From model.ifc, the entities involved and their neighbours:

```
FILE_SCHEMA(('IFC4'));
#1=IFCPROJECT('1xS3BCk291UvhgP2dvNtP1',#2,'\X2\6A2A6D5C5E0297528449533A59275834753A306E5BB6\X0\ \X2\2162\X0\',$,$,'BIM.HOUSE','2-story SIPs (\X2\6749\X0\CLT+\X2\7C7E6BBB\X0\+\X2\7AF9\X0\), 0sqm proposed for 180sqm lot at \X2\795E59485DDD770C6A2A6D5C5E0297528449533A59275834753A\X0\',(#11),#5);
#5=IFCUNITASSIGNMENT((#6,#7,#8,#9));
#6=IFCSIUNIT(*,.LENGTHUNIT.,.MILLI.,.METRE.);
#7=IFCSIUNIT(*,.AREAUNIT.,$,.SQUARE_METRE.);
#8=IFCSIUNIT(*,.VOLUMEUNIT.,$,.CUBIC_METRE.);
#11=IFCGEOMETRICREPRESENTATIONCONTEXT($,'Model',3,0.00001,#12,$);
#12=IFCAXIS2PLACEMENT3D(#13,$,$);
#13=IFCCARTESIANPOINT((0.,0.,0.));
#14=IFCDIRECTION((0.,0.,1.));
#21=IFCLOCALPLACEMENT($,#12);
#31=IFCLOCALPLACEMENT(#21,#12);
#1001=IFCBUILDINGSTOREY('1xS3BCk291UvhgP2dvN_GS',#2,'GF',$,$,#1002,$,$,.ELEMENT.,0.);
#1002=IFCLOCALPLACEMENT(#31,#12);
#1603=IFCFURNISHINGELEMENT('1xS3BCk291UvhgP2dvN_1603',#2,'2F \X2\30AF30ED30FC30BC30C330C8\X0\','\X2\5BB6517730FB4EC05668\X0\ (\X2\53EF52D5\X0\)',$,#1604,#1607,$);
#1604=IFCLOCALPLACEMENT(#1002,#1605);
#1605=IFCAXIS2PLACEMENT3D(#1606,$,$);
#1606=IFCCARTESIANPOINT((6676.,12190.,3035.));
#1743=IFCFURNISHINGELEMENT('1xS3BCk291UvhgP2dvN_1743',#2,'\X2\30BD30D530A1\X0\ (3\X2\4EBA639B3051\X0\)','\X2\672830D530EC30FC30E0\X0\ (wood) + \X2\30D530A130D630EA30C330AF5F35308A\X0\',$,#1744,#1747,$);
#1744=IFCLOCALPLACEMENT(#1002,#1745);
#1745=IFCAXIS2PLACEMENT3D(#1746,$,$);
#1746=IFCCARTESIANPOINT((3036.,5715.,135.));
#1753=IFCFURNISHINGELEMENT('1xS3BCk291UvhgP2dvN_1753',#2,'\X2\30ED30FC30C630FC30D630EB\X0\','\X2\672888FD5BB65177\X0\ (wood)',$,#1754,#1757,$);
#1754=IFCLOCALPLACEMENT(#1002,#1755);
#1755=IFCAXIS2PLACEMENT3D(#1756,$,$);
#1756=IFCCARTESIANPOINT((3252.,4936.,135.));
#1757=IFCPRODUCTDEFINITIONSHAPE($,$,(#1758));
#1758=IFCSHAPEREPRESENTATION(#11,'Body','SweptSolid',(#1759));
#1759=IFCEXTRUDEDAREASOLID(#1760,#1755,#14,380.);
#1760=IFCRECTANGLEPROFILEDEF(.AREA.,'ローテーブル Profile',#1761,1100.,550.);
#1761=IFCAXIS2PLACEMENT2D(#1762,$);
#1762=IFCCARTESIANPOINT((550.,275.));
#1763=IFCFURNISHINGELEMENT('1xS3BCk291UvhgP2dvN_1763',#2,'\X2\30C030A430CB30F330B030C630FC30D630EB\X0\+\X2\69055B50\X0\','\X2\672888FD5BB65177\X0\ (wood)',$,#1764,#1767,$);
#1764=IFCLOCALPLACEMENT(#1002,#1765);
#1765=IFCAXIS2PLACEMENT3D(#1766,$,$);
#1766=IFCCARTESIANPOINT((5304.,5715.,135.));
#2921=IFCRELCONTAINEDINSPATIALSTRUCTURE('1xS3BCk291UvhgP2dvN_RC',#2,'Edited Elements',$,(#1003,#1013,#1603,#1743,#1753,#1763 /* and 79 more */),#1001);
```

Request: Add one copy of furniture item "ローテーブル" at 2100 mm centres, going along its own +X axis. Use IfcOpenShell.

```python
import ifcopenshell
import ifcopenshell.api.geometry
import ifcopenshell.api.root
import ifcopenshell.util.element
import ifcopenshell.util.placement

model = ifcopenshell.open("model.ifc")


def reuse_history(source, copy):
    """copy_class also copies each property set's owner history, people and application; keep the originals."""
    for rel in copy.IsDefinedBy:
        if rel.is_a("IfcRelDefinesByProperties") and (history := rel.RelatingPropertyDefinition.OwnerHistory):
            rel.RelatingPropertyDefinition.OwnerHistory = source.OwnerHistory
            ifcopenshell.util.element.remove_deep2(model, history)


source = model.by_guid("1xS3BCk291UvhgP2dvN_1753")
base = ifcopenshell.util.placement.get_local_placement(source.ObjectPlacement)
step = base[:3, 0] * 2100.0

for i in range(1, 2):
    copy = ifcopenshell.api.root.copy_class(model, product=source)
    copy.Representation = ifcopenshell.util.element.copy_deep(
        model, source.Representation, exclude=["IfcGeometricRepresentationContext", "IfcRepresentationMap"]
    )
    reuse_history(source, copy)
    matrix = base.copy()
    matrix[:3, 3] += i * step
    print("added at", matrix[:3, 3].round(3) + 0.0)
    ifcopenshell.api.geometry.edit_object_placement(model, product=copy, matrix=matrix, is_si=False)

model.write("model_v2.ifc")
```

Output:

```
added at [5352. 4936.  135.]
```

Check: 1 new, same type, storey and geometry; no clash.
